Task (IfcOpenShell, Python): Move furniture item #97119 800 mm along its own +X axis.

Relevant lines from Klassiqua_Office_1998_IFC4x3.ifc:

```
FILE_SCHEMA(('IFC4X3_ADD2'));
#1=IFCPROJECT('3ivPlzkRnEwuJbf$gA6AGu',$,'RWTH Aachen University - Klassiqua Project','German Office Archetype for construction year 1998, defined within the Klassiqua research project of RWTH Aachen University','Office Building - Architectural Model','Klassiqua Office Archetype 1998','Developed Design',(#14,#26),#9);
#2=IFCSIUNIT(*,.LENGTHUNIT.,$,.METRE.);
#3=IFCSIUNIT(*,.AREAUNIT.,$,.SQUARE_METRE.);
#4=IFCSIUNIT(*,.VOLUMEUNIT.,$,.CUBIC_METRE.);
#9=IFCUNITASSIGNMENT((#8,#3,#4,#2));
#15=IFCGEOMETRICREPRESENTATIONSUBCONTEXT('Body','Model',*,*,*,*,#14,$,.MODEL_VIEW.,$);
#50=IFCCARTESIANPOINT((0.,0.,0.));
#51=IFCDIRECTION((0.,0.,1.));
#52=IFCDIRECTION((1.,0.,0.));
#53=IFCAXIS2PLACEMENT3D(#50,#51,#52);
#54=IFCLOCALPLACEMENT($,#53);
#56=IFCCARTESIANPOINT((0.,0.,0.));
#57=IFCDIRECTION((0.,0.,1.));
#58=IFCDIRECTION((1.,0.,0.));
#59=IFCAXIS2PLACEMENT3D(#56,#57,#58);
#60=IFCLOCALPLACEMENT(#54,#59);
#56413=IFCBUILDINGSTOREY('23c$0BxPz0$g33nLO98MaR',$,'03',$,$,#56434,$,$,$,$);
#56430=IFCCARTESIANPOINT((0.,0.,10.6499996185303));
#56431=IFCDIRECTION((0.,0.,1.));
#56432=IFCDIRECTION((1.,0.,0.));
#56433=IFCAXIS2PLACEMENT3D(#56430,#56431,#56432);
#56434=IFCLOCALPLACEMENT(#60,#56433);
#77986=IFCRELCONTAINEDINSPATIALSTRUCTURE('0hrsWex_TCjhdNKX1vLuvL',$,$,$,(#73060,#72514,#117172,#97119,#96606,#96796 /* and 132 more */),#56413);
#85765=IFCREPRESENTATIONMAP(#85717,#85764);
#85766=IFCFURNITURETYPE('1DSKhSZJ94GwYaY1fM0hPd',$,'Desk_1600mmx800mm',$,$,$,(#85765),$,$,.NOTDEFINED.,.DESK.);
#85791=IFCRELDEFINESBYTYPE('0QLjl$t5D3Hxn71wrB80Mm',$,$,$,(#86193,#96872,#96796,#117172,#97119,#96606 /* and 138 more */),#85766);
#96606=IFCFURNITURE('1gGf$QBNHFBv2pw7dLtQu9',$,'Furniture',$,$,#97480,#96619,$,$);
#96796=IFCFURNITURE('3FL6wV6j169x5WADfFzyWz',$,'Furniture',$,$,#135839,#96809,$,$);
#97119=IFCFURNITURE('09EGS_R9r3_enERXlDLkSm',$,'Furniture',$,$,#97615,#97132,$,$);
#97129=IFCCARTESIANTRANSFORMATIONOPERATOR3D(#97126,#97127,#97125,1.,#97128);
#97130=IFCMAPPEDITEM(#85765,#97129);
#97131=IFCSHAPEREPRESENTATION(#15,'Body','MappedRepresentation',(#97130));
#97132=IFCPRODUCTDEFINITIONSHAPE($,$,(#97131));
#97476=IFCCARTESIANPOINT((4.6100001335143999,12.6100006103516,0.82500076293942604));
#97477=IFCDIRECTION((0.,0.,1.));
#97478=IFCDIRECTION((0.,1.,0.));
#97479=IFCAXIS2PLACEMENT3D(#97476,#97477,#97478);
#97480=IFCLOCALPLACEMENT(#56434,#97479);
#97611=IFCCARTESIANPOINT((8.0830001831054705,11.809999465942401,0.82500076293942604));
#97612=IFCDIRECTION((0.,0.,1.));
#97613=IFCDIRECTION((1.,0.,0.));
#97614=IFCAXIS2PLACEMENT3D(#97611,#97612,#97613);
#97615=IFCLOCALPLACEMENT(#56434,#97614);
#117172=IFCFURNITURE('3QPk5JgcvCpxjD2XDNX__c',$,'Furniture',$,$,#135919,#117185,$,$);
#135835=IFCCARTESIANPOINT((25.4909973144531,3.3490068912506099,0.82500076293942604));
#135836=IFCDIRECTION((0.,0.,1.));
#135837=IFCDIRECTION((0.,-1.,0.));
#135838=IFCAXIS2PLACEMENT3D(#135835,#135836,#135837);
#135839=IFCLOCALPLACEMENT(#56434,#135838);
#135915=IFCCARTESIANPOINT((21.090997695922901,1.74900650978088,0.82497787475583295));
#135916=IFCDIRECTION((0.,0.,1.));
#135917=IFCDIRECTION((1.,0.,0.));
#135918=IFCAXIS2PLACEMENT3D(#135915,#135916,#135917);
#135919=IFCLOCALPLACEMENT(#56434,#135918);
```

```python
import ifcopenshell
import ifcopenshell.api.geometry
import ifcopenshell.util.placement

model = ifcopenshell.open("Klassiqua_Office_1998_IFC4x3.ifc")

item = model.by_guid("09EGS_R9r3_enERXlDLkSm")
matrix = ifcopenshell.util.placement.get_local_placement(item.ObjectPlacement)
matrix[:3, 3] += matrix[:3, 0] * 0.8
ifcopenshell.api.geometry.edit_object_placement(model, product=item, matrix=matrix, is_si=False)

print(ifcopenshell.util.placement.get_local_placement(item.ObjectPlacement).round(3) + 0.0)

model.write("Klassiqua_Office_1998_IFC4x3_rev.ifc")
```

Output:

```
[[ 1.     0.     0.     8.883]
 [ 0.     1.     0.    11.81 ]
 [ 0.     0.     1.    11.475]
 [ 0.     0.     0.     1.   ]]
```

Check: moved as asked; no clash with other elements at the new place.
